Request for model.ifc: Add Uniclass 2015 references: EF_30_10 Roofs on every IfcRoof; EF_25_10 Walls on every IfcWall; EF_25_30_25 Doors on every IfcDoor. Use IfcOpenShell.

First a look at what the model holds.

```python
import ifcopenshell

model = ifcopenshell.open("model.ifc")
print(model.schema)
print("classifications:", [c.Name for c in model.by_type("IfcClassification")])
for ifc_class in ("IfcDoor", "IfcRoof", "IfcStair", "IfcWall", "IfcWindow"):
    print(ifc_class, len(model.by_type(ifc_class)))
```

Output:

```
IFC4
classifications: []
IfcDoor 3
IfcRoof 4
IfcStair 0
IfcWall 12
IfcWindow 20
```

```python
import ifcopenshell
import ifcopenshell.api.classification

model = ifcopenshell.open("model.ifc")

system = ifcopenshell.api.classification.add_classification(model, classification="Uniclass 2015")

codes = {
    "IfcRoof": ("EF_30_10", "Roofs"),
    "IfcWall": ("EF_25_10", "Walls"),
    "IfcDoor": ("EF_25_30_25", "Doors"),
}
for ifc_class, (code, name) in codes.items():
    products = model.by_type(ifc_class)
    ifcopenshell.api.classification.add_reference(
        model, products=products, classification=system, identification=code, name=name
    )
    print(code, len(products))

model.write("model_rev.ifc")
```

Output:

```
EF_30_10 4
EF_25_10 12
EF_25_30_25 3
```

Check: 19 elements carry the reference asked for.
